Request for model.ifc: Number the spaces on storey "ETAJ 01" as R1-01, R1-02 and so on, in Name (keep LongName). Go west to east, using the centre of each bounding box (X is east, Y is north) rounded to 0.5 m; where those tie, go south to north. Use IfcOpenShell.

First a look at what the model holds.

```python
import ifcopenshell
import ifcopenshell.util.element
import ifcopenshell.util.placement

model = ifcopenshell.open("model.ifc")
print(model.schema)
storey = next(s for s in model.by_type("IfcBuildingStorey") if s.Name == "ETAJ 01")
spaces = [e for e in ifcopenshell.util.element.get_decomposition(storey) if e.is_a("IfcSpace")]
for e in sorted(spaces, key=lambda e: e.id()):
    origin = ifcopenshell.util.placement.get_local_placement(e.ObjectPlacement)[:3, 3]
    print(e.id(), e.Name, e.LongName, origin.round(2) + 0.0, sep=" | ")
```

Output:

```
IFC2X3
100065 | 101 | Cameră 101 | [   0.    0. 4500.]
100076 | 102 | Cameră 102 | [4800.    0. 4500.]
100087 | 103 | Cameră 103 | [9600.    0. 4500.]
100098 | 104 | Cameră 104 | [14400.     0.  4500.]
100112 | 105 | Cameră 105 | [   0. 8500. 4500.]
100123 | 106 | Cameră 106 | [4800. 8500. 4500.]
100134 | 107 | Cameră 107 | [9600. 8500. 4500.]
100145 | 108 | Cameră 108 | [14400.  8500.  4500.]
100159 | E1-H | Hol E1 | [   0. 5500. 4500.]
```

```python
import ifcopenshell
import ifcopenshell.geom
import ifcopenshell.util.element
import ifcopenshell.util.shape

model = ifcopenshell.open("model.ifc")
settings = ifcopenshell.geom.settings()
settings.set("use-world-coords", True)


def centre(element):
    shape = ifcopenshell.geom.create_shape(settings, element)
    return ifcopenshell.util.shape.get_bbox_centroid(shape.geometry)


storey = next(s for s in model.by_type("IfcBuildingStorey") if s.Name == "ETAJ 01")
spaces = [e for e in ifcopenshell.util.element.get_decomposition(storey) if e.is_a("IfcSpace")]

# Insertion points can sit at a corner or the storey origin, so sort by the geometry (in metres).
centres = {e: centre(e) for e in spaces}
spaces.sort(key=lambda e: (round(centres[e][0] / 0.5), centres[e][1]))

for i, e in enumerate(spaces, start=1):
    number = f"R1-{i:02d}"
    e.Name = number
    print(e.id(), number)

model.write("model_updated.ifc")
```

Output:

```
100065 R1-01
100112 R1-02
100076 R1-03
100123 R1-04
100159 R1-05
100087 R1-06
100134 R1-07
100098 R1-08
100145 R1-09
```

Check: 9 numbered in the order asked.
